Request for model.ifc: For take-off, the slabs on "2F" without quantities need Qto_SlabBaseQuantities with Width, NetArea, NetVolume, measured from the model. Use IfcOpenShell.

First a look at what the model holds.

```python
import ifcopenshell
import ifcopenshell.util.element
import ifcopenshell.util.unit

model = ifcopenshell.open("model.ifc")
print(model.schema)
for unit_type in ("LENGTHUNIT", "AREAUNIT", "VOLUMEUNIT"):
    print(unit_type, ifcopenshell.util.unit.calculate_unit_scale(model, unit_type))
storey = next(s for s in model.by_type("IfcBuildingStorey") if s.Name == "2F")
slabs = [e for e in ifcopenshell.util.element.get_decomposition(storey) if e.is_a("IfcSlab")]
for e in sorted(slabs, key=lambda e: e.id()):
    print(e.id(), e.is_a(), e.Name, list(ifcopenshell.util.element.get_psets(e, qtos_only=True)), sep=" | ")
```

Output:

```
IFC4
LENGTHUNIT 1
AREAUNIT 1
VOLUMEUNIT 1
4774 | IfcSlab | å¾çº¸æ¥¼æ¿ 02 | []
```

```python
import ifcopenshell
import ifcopenshell.api.pset
import ifcopenshell.geom
import ifcopenshell.util.element
import ifcopenshell.util.shape
import ifcopenshell.util.unit

model = ifcopenshell.open("model.ifc")
unit_scale = ifcopenshell.util.unit.calculate_unit_scale(model)
area_scale = ifcopenshell.util.unit.calculate_unit_scale(model, "AREAUNIT")
volume_scale = ifcopenshell.util.unit.calculate_unit_scale(model, "VOLUMEUNIT")
settings = ifcopenshell.geom.settings()

storey = next(s for s in model.by_type("IfcBuildingStorey") if s.Name == "2F")
slabs = [e for e in ifcopenshell.util.element.get_decomposition(storey) if e.is_a("IfcSlab")]

for e in sorted(slabs, key=lambda e: e.id()):
    if ifcopenshell.util.element.get_psets(e, qtos_only=True, should_inherit=False):
        continue
    # Geometry comes back in metres, in the element's own axes.
    shape = ifcopenshell.geom.create_shape(settings, e)
    values = {
        "Width": ifcopenshell.util.shape.get_z(shape.geometry) / unit_scale,
        "NetArea": ifcopenshell.util.shape.get_footprint_area(shape.geometry) / area_scale,
        "NetVolume": ifcopenshell.util.shape.get_volume(shape.geometry) / volume_scale,
    }
    qto = ifcopenshell.api.pset.add_qto(model, product=e, name="Qto_SlabBaseQuantities")
    ifcopenshell.api.pset.edit_qto(model, qto=qto, properties=values)
    print(e.id(), {k: round(v, 3) for k, v in values.items()})

model.write("model_v2.ifc")
```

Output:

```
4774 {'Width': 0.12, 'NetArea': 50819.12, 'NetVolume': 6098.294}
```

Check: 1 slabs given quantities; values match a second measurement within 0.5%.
